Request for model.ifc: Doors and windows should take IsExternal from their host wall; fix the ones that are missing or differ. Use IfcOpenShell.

First a look at what the model holds.

```python
import ifcopenshell
import ifcopenshell.util.element

model = ifcopenshell.open("model.ifc")
print(model.schema)
seen = {}
for e in model.by_type("IfcDoor") + model.by_type("IfcWindow"):
    if not e.FillsVoids:
        continue
    host = e.FillsVoids[0].RelatingOpeningElement.VoidsElements[0].RelatingBuildingElement
    own = ifcopenshell.util.element.get_pset(e, f"Pset_{e.is_a()[3:].removesuffix('StandardCase')}Common", "IsExternal")
    wall = ifcopenshell.util.element.get_pset(host, "Pset_WallCommon", "IsExternal")
    seen[e.is_a(), own, wall] = seen.get((e.is_a(), own, wall), 0) + 1
for (cls, own, wall), count in sorted(seen.items(), key=str):
    print(count, cls, "IsExternal:", own, "| host wall:", wall)
```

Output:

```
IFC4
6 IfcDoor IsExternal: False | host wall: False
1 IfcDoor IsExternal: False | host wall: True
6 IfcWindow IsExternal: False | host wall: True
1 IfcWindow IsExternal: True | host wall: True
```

```python
import ifcopenshell
import ifcopenshell.api.pset
import ifcopenshell.util.element

model = ifcopenshell.open("model.ifc")

count = 0
for ifc_class, pset_name in (("IfcDoor", "Pset_DoorCommon"), ("IfcWindow", "Pset_WindowCommon")):
    for e in model.by_type(ifc_class):
        if not e.FillsVoids:
            continue
        host = e.FillsVoids[0].RelatingOpeningElement.VoidsElements[0].RelatingBuildingElement
        external = ifcopenshell.util.element.get_pset(host, "Pset_WallCommon", "IsExternal")
        if external is None or ifcopenshell.util.element.get_pset(e, pset_name, "IsExternal") == external:
            continue
        pset = ifcopenshell.api.pset.add_pset(model, product=e, name=pset_name)
        ifcopenshell.api.pset.edit_pset(model, pset=pset, properties={"IsExternal": external})
        count += 1

print(count, "updated")

model.write("model-out.ifc")
```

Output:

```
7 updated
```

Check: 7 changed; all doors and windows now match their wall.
